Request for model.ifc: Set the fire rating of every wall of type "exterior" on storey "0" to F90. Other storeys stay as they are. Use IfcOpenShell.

First a look at what the model holds.

```python
import ifcopenshell
import ifcopenshell.util.element

model = ifcopenshell.open("model.ifc")
print(model.schema)
storey = next(s for s in model.by_type("IfcBuildingStorey") if s.Name == "0")
walls = [e for e in ifcopenshell.util.element.get_decomposition(storey) if e.is_a("IfcWall")]
seen = {}
for e in walls:
    element_type = ifcopenshell.util.element.get_type(e)
    key = (element_type.Name if element_type != e and element_type else None, ifcopenshell.util.element.get_pset(e, "Pset_WallCommon", "FireRating"))
    seen[key] = seen.get(key, 0) + 1
for (name, value), count in sorted(seen.items(), key=str):
    print(count, "x", name, "|", value)
```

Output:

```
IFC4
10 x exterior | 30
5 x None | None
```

```python
import ifcopenshell
import ifcopenshell.api.pset
import ifcopenshell.util.element

model = ifcopenshell.open("model.ifc")

storey = next(s for s in model.by_type("IfcBuildingStorey") if s.Name == "0")
walls = [e for e in ifcopenshell.util.element.get_decomposition(storey) if e.is_a("IfcWall")]

count = 0
for e in walls:
    element_type = ifcopenshell.util.element.get_type(e)
    if element_type in (None, e) or element_type.Name != "exterior":
        continue
    # add_pset returns the element's existing set when there is one.
    pset = ifcopenshell.api.pset.add_pset(model, product=e, name="Pset_WallCommon")
    ifcopenshell.api.pset.edit_pset(model, pset=pset, properties={"FireRating": "F90"})
    count += 1

print(count, "walls updated")

model.write("model_updated.ifc")
```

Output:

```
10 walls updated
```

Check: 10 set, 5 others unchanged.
